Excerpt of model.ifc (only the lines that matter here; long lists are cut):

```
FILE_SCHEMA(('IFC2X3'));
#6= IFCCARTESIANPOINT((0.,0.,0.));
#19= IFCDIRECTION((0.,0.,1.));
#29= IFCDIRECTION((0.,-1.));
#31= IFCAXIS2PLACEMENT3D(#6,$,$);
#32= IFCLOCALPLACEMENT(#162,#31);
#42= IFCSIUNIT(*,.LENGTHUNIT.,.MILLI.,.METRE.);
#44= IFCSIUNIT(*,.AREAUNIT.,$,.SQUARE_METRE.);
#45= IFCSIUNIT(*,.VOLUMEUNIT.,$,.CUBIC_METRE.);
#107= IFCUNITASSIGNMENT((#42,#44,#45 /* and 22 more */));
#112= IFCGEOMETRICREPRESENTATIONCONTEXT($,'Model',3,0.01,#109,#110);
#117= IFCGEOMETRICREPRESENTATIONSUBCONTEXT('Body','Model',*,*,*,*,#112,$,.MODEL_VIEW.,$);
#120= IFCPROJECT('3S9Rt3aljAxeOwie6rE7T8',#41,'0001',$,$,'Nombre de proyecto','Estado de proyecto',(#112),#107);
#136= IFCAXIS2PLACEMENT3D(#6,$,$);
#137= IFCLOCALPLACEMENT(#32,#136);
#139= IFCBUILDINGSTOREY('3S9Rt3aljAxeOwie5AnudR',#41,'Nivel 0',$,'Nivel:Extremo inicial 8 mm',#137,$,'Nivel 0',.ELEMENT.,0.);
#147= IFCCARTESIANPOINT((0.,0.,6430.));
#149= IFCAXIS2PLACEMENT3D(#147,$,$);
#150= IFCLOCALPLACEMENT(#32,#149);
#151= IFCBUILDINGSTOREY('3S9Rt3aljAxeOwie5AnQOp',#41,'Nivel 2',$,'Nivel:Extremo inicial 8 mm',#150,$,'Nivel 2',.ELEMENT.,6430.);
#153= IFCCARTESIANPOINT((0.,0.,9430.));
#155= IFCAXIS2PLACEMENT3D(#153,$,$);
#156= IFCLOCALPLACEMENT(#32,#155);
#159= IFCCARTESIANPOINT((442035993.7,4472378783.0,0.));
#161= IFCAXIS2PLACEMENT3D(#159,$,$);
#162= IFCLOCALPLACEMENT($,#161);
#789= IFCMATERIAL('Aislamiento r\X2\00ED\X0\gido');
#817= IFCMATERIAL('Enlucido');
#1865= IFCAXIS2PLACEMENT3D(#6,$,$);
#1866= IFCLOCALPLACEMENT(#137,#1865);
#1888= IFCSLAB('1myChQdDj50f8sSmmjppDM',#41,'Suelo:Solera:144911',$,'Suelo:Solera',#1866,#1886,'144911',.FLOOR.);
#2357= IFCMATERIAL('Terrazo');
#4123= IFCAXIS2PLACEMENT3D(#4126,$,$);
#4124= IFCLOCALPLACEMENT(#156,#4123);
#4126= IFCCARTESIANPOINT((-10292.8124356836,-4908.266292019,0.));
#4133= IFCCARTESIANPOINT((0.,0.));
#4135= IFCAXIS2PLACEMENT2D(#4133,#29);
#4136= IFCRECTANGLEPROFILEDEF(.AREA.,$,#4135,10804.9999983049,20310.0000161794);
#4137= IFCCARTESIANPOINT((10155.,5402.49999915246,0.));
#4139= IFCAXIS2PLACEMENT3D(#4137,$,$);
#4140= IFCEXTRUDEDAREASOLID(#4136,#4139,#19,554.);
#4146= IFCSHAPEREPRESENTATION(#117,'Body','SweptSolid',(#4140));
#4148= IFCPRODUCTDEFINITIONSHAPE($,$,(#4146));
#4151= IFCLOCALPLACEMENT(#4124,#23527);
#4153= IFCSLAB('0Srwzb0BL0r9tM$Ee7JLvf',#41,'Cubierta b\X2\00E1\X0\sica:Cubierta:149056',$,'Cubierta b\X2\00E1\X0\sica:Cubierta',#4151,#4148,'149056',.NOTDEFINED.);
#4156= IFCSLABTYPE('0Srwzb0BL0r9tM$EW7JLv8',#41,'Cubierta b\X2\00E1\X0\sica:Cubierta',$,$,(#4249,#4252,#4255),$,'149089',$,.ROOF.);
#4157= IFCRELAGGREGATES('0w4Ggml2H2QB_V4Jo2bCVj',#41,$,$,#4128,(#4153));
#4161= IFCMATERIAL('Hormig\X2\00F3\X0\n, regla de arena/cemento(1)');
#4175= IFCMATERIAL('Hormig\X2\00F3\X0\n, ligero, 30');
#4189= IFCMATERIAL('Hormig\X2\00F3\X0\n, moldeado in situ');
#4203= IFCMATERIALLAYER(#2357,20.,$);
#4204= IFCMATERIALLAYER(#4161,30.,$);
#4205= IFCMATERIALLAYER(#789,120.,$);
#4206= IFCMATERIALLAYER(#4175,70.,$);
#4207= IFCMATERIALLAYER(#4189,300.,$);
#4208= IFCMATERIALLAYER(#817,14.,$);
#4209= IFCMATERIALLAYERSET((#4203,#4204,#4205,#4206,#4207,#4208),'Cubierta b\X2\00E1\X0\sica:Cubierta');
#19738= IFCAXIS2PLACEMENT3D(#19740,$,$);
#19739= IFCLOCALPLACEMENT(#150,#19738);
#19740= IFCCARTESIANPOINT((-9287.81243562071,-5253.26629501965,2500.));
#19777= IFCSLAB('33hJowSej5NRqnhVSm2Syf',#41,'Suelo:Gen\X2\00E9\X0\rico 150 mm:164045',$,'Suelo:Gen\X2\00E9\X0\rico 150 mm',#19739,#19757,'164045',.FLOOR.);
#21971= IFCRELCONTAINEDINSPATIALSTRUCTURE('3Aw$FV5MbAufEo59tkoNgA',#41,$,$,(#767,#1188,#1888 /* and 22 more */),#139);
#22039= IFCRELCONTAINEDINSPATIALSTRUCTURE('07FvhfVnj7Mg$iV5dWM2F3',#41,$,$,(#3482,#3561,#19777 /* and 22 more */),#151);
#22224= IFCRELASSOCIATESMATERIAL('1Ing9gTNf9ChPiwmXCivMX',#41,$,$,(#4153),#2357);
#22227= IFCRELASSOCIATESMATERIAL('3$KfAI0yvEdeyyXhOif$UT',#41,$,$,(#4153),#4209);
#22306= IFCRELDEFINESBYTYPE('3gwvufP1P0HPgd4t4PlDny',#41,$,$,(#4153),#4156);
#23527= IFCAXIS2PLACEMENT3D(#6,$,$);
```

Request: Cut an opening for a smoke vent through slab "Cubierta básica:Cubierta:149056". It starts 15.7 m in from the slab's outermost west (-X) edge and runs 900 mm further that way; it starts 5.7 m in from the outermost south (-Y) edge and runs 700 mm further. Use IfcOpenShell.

```python
import numpy as np
import ifcopenshell
import ifcopenshell.api.feature
import ifcopenshell.api.geometry
import ifcopenshell.api.root
import ifcopenshell.geom
import ifcopenshell.util.placement
import ifcopenshell.util.representation
import ifcopenshell.util.shape
import ifcopenshell.util.unit

model = ifcopenshell.open("model.ifc")
unit_scale = ifcopenshell.util.unit.calculate_unit_scale(model)
settings = ifcopenshell.geom.settings()


def volume(element):
    """Net volume in cubic metres, openings subtracted."""
    shape = ifcopenshell.geom.create_shape(settings, element)
    return ifcopenshell.util.shape.get_volume(shape.geometry)


slab = model.by_guid("0Srwzb0BL0r9tM$Ee7JLvf")
before = volume(slab)

# Extent in the slab's own axes, in metres. The edges named are its -X and -Y sides.
slab_shape = ifcopenshell.geom.create_shape(settings, slab)
vertices = ifcopenshell.util.shape.get_vertices(slab_shape.geometry)
x_min, y_min, bottom = vertices.min(axis=0)
top = vertices[:, 2].max()

opening = ifcopenshell.api.root.create_entity(model, ifc_class="IfcOpeningElement", name="Smoke vent opening")
context = ifcopenshell.util.representation.get_context(model, "Model", "Body", "MODEL_VIEW")
width, depth = 0.9, 0.7
outline = [(0.0, 0.0), (width, 0.0), (width, depth), (0.0, depth), (0.0, 0.0)]
# Overshoot both faces by 50 mm so the cut is clean.
shape = ifcopenshell.api.geometry.add_slab_representation(
    model, context=context, depth=top - bottom + 0.1, polyline=outline
)
ifcopenshell.api.geometry.assign_representation(model, product=opening, representation=shape)

matrix = ifcopenshell.util.placement.get_local_placement(slab.ObjectPlacement)
matrix[:, 3] = matrix @ np.append(np.array([x_min + 15.7, y_min + 5.7, bottom - 0.05]) / unit_scale, 1.0)
ifcopenshell.api.geometry.edit_object_placement(model, product=opening, matrix=matrix, is_si=False)
ifcopenshell.api.feature.add_feature(model, feature=opening, element=slab)

after = volume(slab)

print(f"slab volume {before:.3f} -> {after:.3f} m3")

model.write("model-out.ifc")
```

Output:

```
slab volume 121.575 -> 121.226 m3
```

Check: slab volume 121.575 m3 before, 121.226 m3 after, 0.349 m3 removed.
